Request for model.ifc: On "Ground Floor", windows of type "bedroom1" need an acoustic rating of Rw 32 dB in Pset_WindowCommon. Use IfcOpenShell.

First a look at what the model holds.

```python
import ifcopenshell
import ifcopenshell.util.element

model = ifcopenshell.open("model.ifc")
print(model.schema)
storey = next(s for s in model.by_type("IfcBuildingStorey") if s.Name == "Ground Floor")
windows = [e for e in ifcopenshell.util.element.get_decomposition(storey) if e.is_a("IfcWindow")]
seen = {}
for e in windows:
    element_type = ifcopenshell.util.element.get_type(e)
    key = (element_type.Name if element_type != e and element_type else None, ifcopenshell.util.element.get_pset(e, "Pset_WindowCommon", "AcousticRating"))
    seen[key] = seen.get(key, 0) + 1
for (name, value), count in sorted(seen.items(), key=str):
    print(count, "x", name, "|", value)
```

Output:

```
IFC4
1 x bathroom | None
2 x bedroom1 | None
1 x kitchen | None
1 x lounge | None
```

```python
import ifcopenshell
import ifcopenshell.api.pset
import ifcopenshell.util.element

model = ifcopenshell.open("model.ifc")

storey = next(s for s in model.by_type("IfcBuildingStorey") if s.Name == "Ground Floor")
windows = [e for e in ifcopenshell.util.element.get_decomposition(storey) if e.is_a("IfcWindow")]

count = 0
for e in windows:
    element_type = ifcopenshell.util.element.get_type(e)
    if element_type in (None, e) or element_type.Name != "bedroom1":
        continue
    # add_pset returns the element's existing set when there is one.
    pset = ifcopenshell.api.pset.add_pset(model, product=e, name="Pset_WindowCommon")
    ifcopenshell.api.pset.edit_pset(model, pset=pset, properties={"AcousticRating": "Rw 32 dB"})
    count += 1

print(count, "windows updated")

model.write("model-out.ifc")
```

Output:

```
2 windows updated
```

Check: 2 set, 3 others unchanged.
